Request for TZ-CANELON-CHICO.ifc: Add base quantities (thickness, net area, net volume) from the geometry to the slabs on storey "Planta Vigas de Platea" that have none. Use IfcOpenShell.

First a look at what the model holds.

```python
import ifcopenshell
import ifcopenshell.util.element
import ifcopenshell.util.unit

model = ifcopenshell.open("TZ-CANELON-CHICO.ifc")
print(model.schema)
for unit_type in ("LENGTHUNIT", "AREAUNIT", "VOLUMEUNIT"):
    print(unit_type, ifcopenshell.util.unit.calculate_unit_scale(model, unit_type))
storey = next(s for s in model.by_type("IfcBuildingStorey") if s.Name == "Planta Vigas de Platea")
slabs = [e for e in ifcopenshell.util.element.get_decomposition(storey) if e.is_a("IfcSlab")]
for e in sorted(slabs, key=lambda e: e.id()):
    print(e.id(), e.is_a(), e.Name, list(ifcopenshell.util.element.get_psets(e, qtos_only=True)), sep=" | ")
```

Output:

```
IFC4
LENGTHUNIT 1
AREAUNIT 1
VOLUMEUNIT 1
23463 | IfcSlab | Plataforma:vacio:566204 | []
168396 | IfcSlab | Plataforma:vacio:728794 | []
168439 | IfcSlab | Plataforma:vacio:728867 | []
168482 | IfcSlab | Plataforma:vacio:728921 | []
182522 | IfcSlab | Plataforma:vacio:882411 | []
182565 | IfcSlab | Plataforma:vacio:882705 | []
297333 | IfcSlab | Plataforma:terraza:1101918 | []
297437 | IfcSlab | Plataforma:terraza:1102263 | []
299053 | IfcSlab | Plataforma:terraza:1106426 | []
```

```python
import ifcopenshell
import ifcopenshell.api.pset
import ifcopenshell.geom
import ifcopenshell.util.element
import ifcopenshell.util.shape
import ifcopenshell.util.unit

model = ifcopenshell.open("TZ-CANELON-CHICO.ifc")
unit_scale = ifcopenshell.util.unit.calculate_unit_scale(model)
area_scale = ifcopenshell.util.unit.calculate_unit_scale(model, "AREAUNIT")
volume_scale = ifcopenshell.util.unit.calculate_unit_scale(model, "VOLUMEUNIT")
settings = ifcopenshell.geom.settings()

storey = next(s for s in model.by_type("IfcBuildingStorey") if s.Name == "Planta Vigas de Platea")
slabs = [e for e in ifcopenshell.util.element.get_decomposition(storey) if e.is_a("IfcSlab")]

for e in sorted(slabs, key=lambda e: e.id()):
    if ifcopenshell.util.element.get_psets(e, qtos_only=True, should_inherit=False):
        continue
    # Geometry comes back in metres, in the element's own axes.
    shape = ifcopenshell.geom.create_shape(settings, e)
    values = {
        "Width": ifcopenshell.util.shape.get_z(shape.geometry) / unit_scale,
        "NetArea": ifcopenshell.util.shape.get_footprint_area(shape.geometry) / area_scale,
        "NetVolume": ifcopenshell.util.shape.get_volume(shape.geometry) / volume_scale,
    }
    qto = ifcopenshell.api.pset.add_qto(model, product=e, name="Qto_SlabBaseQuantities")
    ifcopenshell.api.pset.edit_qto(model, qto=qto, properties=values)
    print(e.id(), {k: round(v, 3) for k, v in values.items()})

model.write("TZ-CANELON-CHICO-out.ifc")
```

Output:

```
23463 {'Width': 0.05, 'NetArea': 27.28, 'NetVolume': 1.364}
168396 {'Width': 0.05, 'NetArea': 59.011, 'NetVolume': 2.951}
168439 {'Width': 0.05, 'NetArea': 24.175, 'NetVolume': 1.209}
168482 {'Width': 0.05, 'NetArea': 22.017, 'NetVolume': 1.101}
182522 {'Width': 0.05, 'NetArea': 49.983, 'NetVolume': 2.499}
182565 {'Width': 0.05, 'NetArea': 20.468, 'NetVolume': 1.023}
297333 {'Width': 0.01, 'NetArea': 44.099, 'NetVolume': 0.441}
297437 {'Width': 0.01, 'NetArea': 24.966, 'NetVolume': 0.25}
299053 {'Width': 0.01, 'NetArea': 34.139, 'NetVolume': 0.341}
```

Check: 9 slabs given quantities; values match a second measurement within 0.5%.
